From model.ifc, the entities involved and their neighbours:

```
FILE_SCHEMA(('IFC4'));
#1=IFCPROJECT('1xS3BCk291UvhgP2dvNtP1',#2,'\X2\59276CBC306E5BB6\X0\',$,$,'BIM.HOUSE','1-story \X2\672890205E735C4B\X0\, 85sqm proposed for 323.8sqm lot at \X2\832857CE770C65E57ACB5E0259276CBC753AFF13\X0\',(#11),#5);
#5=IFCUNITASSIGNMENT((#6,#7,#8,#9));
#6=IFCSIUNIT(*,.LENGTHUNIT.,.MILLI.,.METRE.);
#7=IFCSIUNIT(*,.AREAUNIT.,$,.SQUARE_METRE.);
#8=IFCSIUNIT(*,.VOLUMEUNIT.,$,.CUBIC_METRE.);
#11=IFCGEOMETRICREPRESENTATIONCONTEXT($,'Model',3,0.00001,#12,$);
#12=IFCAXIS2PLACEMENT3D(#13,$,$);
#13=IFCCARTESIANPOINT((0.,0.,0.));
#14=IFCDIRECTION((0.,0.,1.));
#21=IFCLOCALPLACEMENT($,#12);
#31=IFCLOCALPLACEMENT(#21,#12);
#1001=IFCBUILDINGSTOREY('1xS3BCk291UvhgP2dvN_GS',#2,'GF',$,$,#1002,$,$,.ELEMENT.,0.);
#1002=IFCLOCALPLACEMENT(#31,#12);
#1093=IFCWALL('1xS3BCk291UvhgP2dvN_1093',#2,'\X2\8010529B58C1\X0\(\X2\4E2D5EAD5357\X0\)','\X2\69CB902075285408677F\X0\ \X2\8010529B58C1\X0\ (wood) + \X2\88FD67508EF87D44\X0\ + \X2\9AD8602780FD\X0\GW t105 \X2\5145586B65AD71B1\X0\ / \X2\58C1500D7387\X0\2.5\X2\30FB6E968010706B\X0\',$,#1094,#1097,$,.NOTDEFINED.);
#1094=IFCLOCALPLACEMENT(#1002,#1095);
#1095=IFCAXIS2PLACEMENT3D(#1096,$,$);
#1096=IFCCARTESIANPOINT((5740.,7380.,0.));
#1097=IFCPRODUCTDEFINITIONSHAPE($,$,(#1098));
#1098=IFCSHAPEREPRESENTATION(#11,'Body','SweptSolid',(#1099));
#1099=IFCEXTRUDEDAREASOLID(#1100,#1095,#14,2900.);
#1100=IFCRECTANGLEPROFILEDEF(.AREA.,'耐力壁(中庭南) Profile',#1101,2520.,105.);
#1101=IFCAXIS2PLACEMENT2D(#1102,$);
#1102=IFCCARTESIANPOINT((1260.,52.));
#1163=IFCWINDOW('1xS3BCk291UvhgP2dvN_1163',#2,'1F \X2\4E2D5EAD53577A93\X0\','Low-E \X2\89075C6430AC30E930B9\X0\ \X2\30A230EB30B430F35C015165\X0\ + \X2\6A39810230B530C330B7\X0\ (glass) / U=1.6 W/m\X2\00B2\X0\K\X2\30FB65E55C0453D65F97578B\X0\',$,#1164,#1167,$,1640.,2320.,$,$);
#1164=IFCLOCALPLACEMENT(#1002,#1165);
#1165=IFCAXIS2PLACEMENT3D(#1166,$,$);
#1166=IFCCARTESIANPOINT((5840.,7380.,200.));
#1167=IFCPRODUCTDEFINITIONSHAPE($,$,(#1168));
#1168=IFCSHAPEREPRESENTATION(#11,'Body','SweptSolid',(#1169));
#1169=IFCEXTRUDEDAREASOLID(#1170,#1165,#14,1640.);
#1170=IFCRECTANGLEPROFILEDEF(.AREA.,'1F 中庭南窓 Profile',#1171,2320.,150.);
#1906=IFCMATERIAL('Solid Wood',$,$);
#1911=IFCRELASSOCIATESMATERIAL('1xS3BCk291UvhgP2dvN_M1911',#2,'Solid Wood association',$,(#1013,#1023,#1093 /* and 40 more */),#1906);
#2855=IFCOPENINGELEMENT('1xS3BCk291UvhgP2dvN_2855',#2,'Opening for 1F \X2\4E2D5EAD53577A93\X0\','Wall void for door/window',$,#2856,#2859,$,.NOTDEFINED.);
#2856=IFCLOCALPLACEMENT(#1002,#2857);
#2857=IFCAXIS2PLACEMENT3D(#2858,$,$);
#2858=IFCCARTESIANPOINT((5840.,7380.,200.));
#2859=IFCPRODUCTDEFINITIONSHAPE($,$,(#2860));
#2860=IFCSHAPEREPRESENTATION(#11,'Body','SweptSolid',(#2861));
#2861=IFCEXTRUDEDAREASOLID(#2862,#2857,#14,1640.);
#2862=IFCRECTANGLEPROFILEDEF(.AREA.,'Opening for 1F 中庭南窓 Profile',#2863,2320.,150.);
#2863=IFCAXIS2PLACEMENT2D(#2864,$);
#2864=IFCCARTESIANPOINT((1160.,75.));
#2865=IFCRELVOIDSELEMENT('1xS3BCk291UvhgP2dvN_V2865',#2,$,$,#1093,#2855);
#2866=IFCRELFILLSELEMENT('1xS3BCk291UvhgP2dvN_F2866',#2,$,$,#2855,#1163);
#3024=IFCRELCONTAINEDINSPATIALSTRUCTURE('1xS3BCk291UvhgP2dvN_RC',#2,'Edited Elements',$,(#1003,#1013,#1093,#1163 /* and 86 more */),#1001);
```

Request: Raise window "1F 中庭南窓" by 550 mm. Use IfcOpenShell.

```python
import numpy as np
import ifcopenshell
import ifcopenshell.api.geometry
import ifcopenshell.util.placement
import ifcopenshell.util.unit

model = ifcopenshell.open("model.ifc")
unit_scale = ifcopenshell.util.unit.calculate_unit_scale(model)

window = model.by_guid("1xS3BCk291UvhgP2dvN_1163")
opening = window.FillsVoids[0].RelatingOpeningElement
dz = 550.0

shift = np.array([0.0, 0.0, dz])
# The window is not placed relative to its opening, so move both.
for product in (opening, window):
    matrix = ifcopenshell.util.placement.get_local_placement(product.ObjectPlacement)
    matrix[:3, 3] += shift
    ifcopenshell.api.geometry.edit_object_placement(model, product=product, matrix=matrix, is_si=False)

print(f"moved by {dz * unit_scale:+.3f} m")

model.write("model_edited.ifc")
```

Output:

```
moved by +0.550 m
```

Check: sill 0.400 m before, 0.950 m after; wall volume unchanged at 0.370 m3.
